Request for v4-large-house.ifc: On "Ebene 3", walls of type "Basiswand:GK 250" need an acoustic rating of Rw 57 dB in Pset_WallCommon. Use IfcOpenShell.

First a look at what the model holds.

```python
import ifcopenshell
import ifcopenshell.util.element

model = ifcopenshell.open("v4-large-house.ifc")
print(model.schema)
storey = next(s for s in model.by_type("IfcBuildingStorey") if s.Name == "Ebene 3")
walls = [e for e in ifcopenshell.util.element.get_decomposition(storey) if e.is_a("IfcWall")]
seen = {}
for e in walls:
    element_type = ifcopenshell.util.element.get_type(e)
    key = (element_type.Name if element_type != e and element_type else None, ifcopenshell.util.element.get_pset(e, "Pset_WallCommon", "AcousticRating"))
    seen[key] = seen.get(key, 0) + 1
for (name, value), count in sorted(seen.items(), key=str):
    print(count, "x", name, "|", value)
```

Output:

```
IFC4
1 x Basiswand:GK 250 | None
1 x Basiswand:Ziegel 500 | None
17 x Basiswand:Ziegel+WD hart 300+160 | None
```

```python
import ifcopenshell
import ifcopenshell.api.pset
import ifcopenshell.util.element

model = ifcopenshell.open("v4-large-house.ifc")

storey = next(s for s in model.by_type("IfcBuildingStorey") if s.Name == "Ebene 3")
walls = [e for e in ifcopenshell.util.element.get_decomposition(storey) if e.is_a("IfcWall")]

count = 0
for e in walls:
    element_type = ifcopenshell.util.element.get_type(e)
    if element_type in (None, e) or element_type.Name != "Basiswand:GK 250":
        continue
    # add_pset returns the element's existing set when there is one.
    pset = ifcopenshell.api.pset.add_pset(model, product=e, name="Pset_WallCommon")
    ifcopenshell.api.pset.edit_pset(model, pset=pset, properties={"AcousticRating": "Rw 57 dB"})
    count += 1

print(count, "walls updated")

model.write("v4-large-house_edited.ifc")
```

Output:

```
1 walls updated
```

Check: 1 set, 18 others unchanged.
